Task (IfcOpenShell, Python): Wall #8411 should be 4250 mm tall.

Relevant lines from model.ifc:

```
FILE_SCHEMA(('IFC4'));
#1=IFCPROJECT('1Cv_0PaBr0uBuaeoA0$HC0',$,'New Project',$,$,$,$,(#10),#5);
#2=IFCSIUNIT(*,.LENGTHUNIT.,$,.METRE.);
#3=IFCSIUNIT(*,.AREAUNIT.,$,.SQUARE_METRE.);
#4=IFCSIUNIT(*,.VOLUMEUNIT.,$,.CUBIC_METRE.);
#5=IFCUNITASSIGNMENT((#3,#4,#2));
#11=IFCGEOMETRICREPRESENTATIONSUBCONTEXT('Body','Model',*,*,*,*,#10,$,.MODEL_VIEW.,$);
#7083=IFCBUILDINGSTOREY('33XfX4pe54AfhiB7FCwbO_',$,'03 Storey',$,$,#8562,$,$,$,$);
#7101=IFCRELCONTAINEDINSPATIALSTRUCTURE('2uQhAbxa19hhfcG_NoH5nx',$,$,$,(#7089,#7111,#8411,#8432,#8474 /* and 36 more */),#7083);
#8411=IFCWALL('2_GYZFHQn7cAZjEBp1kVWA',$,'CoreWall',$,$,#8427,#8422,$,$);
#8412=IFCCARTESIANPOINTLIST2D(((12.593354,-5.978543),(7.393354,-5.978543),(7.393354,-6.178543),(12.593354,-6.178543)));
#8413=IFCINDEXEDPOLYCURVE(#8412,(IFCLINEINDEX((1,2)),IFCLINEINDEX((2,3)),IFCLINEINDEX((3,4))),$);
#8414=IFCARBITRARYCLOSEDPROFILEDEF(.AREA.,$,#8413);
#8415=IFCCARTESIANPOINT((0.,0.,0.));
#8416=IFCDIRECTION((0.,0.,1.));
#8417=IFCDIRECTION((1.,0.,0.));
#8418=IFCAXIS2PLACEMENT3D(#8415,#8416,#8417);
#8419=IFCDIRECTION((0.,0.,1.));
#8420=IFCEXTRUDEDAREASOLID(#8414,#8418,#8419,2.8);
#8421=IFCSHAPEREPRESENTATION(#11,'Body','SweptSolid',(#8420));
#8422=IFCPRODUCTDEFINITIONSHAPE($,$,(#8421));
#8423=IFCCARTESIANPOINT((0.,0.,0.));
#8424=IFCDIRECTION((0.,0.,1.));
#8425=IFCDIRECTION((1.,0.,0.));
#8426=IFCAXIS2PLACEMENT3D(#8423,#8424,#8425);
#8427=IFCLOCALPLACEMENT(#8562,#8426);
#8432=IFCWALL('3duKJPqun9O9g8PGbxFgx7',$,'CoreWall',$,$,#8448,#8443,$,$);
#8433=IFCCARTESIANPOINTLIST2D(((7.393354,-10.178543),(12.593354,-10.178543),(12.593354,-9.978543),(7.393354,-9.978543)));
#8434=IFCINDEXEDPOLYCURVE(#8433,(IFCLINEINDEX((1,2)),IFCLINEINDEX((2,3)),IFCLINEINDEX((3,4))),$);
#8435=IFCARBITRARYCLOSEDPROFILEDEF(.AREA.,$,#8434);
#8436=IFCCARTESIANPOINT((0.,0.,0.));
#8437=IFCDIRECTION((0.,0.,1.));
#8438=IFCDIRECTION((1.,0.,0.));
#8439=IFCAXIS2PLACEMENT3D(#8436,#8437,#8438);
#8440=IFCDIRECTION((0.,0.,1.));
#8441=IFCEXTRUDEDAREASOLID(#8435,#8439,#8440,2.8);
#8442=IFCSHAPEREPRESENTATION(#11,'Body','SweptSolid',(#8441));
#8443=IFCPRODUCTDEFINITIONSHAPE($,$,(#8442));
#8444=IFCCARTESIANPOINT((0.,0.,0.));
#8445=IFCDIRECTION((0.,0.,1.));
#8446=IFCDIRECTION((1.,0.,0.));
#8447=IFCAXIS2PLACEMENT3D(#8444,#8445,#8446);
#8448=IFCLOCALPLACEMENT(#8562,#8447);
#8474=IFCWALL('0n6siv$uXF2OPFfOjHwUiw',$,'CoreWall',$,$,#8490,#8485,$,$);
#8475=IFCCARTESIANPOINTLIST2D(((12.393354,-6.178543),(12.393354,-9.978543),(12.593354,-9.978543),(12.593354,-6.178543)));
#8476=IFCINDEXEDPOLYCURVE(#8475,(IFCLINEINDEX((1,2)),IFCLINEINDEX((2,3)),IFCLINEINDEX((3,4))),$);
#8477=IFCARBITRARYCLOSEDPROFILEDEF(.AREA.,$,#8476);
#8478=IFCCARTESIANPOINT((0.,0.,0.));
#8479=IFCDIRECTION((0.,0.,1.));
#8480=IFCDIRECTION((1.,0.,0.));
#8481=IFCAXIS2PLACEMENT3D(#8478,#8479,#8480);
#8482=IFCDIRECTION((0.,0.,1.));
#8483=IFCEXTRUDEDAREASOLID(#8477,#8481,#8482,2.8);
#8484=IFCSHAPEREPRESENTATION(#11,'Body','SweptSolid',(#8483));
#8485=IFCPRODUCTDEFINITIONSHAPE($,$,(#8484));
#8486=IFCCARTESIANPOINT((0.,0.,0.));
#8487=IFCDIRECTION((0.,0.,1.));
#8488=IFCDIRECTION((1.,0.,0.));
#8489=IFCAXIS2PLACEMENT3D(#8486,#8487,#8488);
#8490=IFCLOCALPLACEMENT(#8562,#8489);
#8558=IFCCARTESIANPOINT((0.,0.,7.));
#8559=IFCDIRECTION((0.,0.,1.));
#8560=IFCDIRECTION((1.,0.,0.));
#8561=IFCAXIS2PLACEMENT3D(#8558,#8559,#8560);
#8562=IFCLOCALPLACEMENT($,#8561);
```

```python
import ifcopenshell
import ifcopenshell.geom
import ifcopenshell.util.representation
import ifcopenshell.util.shape
import ifcopenshell.util.unit

model = ifcopenshell.open("model.ifc")
unit_scale = ifcopenshell.util.unit.calculate_unit_scale(model)
settings = ifcopenshell.geom.settings()


def volume(element):
    """Net volume in cubic metres, openings subtracted."""
    shape = ifcopenshell.geom.create_shape(settings, element)
    return ifcopenshell.util.shape.get_volume(shape.geometry)


wall = model.by_guid("2_GYZFHQn7cAZjEBp1kVWA")
before = volume(wall)

body = ifcopenshell.util.representation.get_representation(wall, "Model", "Body")
solid = body.Items[0]
old_height = solid.Depth
solid.Depth = 4.25 / unit_scale
after = volume(wall)

print(f"height {old_height:g} -> {solid.Depth:g}, volume {before:.3f} -> {after:.3f} m3")

model.write("model_edited.ifc")
```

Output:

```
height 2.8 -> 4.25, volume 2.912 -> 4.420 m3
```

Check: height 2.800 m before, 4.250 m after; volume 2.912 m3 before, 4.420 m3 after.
